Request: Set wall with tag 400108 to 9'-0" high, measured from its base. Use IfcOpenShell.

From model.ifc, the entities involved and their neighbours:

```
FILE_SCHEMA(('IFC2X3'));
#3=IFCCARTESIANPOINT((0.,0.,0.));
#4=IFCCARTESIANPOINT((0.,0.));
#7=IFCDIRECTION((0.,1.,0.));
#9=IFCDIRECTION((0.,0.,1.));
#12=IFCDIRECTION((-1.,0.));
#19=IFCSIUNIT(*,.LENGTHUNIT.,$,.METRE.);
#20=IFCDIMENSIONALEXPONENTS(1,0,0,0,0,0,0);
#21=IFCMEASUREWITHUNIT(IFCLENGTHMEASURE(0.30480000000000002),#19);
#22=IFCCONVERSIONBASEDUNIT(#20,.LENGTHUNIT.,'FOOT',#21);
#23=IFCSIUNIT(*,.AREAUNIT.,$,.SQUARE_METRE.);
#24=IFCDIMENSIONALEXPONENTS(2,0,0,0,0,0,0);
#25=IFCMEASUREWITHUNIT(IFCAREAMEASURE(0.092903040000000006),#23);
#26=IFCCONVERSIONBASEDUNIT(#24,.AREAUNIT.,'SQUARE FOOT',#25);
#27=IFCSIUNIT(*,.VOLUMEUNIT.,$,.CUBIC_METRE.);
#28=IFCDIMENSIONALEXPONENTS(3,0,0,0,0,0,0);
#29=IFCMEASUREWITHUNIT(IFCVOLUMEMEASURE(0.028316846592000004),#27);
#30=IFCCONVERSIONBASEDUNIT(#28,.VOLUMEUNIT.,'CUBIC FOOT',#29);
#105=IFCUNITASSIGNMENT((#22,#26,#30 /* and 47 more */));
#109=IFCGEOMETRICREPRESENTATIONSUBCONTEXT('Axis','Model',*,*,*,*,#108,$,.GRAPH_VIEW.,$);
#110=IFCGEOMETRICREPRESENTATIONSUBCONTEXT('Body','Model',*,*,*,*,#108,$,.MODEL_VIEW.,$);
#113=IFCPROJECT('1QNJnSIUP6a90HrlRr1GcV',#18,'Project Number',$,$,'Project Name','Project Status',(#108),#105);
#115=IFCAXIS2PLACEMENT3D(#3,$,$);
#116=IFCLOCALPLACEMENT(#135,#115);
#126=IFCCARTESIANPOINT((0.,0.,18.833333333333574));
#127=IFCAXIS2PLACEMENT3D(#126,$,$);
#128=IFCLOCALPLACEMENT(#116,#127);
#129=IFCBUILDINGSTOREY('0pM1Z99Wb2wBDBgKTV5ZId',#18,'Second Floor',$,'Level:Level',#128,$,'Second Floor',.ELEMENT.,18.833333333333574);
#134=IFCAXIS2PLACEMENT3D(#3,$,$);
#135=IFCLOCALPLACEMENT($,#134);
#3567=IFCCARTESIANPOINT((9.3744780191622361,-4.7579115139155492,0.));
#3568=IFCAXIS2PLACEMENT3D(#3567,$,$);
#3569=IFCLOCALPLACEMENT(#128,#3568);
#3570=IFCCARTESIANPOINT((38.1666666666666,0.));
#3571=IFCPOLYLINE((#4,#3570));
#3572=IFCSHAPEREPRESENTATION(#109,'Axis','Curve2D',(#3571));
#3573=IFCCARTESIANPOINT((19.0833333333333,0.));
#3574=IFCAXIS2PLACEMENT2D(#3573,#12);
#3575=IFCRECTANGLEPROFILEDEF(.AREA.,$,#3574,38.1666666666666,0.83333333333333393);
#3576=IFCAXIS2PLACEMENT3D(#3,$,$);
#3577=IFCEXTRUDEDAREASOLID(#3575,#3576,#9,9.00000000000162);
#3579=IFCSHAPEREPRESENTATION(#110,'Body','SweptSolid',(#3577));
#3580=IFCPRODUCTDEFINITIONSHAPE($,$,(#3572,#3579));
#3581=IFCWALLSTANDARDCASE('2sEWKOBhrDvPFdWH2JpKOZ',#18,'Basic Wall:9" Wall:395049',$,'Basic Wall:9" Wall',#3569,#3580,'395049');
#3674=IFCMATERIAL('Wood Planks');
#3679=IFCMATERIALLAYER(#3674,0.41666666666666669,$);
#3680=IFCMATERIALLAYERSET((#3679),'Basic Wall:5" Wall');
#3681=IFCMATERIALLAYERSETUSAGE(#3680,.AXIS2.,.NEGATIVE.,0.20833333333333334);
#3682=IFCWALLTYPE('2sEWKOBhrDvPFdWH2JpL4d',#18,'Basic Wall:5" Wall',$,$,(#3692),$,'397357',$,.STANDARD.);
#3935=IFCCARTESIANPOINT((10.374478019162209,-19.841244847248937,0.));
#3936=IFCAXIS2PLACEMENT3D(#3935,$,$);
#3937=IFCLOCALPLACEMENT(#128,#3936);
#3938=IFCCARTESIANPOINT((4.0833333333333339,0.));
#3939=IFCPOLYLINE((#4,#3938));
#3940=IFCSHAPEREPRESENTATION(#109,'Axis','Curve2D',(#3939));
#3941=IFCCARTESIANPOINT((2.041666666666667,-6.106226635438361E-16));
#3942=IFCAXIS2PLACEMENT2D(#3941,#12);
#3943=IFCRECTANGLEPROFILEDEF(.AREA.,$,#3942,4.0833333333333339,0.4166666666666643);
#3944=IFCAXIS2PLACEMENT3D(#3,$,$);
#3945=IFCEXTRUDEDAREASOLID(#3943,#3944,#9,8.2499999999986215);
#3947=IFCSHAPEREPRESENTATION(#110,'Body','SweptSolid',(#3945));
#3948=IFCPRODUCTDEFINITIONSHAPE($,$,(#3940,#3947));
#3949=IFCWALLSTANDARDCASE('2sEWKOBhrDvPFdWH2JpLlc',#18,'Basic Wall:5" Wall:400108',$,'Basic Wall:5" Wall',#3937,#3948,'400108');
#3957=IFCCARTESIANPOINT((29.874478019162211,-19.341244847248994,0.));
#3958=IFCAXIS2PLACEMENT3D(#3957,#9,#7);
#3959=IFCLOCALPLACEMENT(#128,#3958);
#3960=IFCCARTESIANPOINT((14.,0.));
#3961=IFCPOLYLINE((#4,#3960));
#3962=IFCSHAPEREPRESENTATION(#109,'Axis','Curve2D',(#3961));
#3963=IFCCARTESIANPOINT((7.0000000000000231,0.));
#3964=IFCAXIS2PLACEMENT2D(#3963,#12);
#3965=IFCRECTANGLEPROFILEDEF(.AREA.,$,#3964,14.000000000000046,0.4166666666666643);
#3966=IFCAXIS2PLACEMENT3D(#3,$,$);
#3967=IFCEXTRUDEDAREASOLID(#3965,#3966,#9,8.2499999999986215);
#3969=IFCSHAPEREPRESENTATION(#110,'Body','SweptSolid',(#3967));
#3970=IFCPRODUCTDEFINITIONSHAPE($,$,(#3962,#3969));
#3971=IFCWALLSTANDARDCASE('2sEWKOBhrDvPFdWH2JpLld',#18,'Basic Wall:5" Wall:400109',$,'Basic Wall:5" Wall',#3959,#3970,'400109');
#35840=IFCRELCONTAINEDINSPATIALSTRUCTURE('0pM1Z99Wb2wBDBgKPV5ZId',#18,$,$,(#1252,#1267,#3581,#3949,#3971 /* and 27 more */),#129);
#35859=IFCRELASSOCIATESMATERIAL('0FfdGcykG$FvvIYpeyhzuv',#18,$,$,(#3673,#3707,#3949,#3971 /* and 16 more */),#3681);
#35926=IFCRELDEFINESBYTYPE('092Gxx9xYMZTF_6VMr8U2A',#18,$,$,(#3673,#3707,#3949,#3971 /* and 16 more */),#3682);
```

```python
import ifcopenshell
import ifcopenshell.geom
import ifcopenshell.util.representation
import ifcopenshell.util.shape
import ifcopenshell.util.unit

model = ifcopenshell.open("model.ifc")
unit_scale = ifcopenshell.util.unit.calculate_unit_scale(model)
settings = ifcopenshell.geom.settings()


def volume(element):
    """Net volume in cubic metres, openings subtracted."""
    shape = ifcopenshell.geom.create_shape(settings, element)
    return ifcopenshell.util.shape.get_volume(shape.geometry)


wall = model.by_id(3949)
before = volume(wall)

body = ifcopenshell.util.representation.get_representation(wall, "Model", "Body")
solid = body.Items[0]
old_height = solid.Depth
solid.Depth = 108 * 0.0254 / unit_scale
after = volume(wall)

print(f"height {old_height:g} -> {solid.Depth:g}, volume {before:.3f} -> {after:.3f} m3")

model.write("model_rev.ifc")
```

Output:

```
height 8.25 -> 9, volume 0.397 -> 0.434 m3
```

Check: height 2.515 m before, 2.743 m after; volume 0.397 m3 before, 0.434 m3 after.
